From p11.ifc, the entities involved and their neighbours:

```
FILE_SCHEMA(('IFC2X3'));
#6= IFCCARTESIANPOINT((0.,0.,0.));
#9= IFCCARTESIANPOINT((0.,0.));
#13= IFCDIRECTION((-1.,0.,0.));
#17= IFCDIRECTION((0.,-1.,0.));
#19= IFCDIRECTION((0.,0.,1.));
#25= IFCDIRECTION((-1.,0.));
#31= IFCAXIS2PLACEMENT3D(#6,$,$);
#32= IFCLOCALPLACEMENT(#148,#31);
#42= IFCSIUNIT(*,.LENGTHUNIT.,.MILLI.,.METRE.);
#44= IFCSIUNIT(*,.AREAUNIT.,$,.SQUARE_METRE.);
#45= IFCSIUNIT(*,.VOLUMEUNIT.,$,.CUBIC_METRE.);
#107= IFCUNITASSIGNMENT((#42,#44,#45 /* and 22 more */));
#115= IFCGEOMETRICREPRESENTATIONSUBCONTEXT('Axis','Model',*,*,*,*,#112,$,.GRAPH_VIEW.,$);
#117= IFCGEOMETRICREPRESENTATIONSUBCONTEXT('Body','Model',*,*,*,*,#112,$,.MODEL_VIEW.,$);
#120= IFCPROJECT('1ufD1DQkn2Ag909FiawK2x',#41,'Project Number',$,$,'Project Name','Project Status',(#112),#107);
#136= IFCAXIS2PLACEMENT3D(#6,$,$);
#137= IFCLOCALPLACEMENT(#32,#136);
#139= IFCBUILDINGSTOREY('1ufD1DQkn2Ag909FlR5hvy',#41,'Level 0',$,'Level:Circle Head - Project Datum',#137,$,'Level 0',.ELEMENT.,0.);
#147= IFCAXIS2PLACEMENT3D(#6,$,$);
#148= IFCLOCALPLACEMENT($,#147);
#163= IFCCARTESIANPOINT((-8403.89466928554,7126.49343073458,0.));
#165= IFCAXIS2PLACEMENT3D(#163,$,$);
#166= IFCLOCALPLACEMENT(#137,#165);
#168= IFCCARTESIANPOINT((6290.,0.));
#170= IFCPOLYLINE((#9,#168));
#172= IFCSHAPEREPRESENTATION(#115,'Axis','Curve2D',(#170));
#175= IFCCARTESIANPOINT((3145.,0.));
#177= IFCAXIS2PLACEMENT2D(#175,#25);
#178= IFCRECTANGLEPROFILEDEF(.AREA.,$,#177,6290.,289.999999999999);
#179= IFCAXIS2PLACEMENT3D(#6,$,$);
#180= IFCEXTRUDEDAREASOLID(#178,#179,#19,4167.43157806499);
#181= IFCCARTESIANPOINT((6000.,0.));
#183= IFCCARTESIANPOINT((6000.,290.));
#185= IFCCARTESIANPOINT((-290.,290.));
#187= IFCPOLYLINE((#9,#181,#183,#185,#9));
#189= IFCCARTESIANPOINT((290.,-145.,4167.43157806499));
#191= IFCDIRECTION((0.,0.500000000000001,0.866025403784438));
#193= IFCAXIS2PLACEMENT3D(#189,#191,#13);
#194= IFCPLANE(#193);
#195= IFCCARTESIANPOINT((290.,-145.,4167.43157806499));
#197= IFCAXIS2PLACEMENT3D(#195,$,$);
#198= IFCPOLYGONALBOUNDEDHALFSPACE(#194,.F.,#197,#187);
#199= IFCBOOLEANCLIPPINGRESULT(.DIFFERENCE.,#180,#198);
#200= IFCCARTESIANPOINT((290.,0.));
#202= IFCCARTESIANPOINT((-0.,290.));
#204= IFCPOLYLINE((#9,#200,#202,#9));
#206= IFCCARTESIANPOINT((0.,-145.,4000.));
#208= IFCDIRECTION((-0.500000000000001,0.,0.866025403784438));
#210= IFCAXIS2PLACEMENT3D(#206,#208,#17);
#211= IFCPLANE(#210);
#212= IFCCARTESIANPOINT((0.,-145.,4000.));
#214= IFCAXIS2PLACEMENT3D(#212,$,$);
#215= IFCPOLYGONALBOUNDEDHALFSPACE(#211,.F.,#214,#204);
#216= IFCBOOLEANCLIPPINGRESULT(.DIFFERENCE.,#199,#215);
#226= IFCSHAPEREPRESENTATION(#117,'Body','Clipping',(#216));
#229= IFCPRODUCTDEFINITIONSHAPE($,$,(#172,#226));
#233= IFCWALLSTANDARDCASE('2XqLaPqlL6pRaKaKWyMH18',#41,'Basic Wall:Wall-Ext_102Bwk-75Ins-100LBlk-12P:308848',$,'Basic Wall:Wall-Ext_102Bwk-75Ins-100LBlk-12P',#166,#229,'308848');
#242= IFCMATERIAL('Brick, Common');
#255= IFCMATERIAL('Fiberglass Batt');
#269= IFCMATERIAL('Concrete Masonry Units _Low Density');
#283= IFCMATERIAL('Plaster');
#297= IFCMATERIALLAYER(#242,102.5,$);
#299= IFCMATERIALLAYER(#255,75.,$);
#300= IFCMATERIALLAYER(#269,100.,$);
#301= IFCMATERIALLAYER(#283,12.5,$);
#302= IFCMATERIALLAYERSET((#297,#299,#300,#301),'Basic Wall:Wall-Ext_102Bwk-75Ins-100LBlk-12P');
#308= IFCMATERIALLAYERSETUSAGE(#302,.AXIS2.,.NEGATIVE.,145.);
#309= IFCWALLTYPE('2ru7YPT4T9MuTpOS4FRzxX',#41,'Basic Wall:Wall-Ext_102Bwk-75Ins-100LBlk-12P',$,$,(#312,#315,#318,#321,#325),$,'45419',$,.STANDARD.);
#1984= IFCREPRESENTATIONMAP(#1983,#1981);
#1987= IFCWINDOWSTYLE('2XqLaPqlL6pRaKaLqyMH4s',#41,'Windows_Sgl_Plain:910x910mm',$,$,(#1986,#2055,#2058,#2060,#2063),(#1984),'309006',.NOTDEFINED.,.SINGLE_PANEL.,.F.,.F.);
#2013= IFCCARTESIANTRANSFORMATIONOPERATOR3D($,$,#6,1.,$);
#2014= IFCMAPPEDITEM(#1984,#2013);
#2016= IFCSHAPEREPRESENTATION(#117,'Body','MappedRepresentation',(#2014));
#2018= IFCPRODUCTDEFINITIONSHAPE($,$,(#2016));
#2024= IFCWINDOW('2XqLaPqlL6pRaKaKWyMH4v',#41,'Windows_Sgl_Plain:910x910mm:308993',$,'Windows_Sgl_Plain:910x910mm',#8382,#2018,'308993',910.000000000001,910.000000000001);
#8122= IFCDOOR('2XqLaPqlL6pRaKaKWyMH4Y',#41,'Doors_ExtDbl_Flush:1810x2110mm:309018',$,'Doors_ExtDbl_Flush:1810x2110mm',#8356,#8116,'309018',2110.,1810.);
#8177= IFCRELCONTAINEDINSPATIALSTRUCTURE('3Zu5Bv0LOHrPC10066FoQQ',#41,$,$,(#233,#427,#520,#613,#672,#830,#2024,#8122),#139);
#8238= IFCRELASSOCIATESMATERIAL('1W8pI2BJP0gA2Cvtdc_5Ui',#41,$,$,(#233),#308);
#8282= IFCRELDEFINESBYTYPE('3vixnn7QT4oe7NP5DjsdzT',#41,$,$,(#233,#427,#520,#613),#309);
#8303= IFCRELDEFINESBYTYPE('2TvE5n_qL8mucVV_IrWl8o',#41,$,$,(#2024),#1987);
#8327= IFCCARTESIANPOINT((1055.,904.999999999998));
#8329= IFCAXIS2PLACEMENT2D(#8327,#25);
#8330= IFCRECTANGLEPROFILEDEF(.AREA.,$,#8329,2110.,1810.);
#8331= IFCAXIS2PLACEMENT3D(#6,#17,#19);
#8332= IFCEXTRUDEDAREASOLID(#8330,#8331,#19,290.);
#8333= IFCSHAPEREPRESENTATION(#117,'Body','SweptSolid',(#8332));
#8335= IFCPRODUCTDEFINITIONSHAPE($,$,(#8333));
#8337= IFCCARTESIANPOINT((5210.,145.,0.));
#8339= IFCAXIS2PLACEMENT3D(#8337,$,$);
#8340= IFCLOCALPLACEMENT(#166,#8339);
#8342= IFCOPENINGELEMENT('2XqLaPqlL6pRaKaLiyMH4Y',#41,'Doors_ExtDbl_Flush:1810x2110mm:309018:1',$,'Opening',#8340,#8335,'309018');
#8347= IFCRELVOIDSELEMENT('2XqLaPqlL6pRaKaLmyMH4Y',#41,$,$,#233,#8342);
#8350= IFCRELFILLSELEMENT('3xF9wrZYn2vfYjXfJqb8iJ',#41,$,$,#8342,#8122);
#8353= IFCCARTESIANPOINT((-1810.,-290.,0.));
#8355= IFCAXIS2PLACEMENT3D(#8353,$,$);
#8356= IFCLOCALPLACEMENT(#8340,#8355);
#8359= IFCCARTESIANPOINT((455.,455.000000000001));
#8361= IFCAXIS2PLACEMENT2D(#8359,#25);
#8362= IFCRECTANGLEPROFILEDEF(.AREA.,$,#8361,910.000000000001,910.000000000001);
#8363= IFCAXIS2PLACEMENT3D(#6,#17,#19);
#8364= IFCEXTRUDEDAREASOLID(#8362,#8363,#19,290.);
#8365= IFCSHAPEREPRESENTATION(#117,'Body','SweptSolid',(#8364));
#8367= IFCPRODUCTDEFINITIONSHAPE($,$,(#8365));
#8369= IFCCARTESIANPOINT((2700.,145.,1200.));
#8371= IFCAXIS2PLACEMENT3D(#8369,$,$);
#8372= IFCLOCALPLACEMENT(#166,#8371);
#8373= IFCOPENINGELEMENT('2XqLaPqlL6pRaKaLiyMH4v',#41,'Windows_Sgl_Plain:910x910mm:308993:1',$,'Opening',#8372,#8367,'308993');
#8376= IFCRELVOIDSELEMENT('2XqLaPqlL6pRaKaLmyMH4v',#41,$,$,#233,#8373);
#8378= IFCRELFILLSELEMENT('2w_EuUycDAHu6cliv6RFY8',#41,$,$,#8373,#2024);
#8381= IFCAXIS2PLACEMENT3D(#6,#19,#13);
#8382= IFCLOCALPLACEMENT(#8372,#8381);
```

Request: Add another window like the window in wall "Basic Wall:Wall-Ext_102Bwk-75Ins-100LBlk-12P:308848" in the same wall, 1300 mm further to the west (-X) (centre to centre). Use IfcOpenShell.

```python
import ifcopenshell
import ifcopenshell.api.feature
import ifcopenshell.api.geometry
import ifcopenshell.api.root
import ifcopenshell.geom
import ifcopenshell.util.element
import ifcopenshell.util.placement
import ifcopenshell.util.shape
import ifcopenshell.util.unit

model = ifcopenshell.open("p11.ifc")
unit_scale = ifcopenshell.util.unit.calculate_unit_scale(model)
settings = ifcopenshell.geom.settings()


def volume(element):
    """Net volume in cubic metres, openings subtracted."""
    shape = ifcopenshell.geom.create_shape(settings, element)
    return ifcopenshell.util.shape.get_volume(shape.geometry)


def reuse_history(source, copy):
    """copy_class also copies each property set's owner history, people and application; keep the originals."""
    for rel in copy.IsDefinedBy:
        if rel.is_a("IfcRelDefinesByProperties") and (history := rel.RelatingPropertyDefinition.OwnerHistory):
            rel.RelatingPropertyDefinition.OwnerHistory = source.OwnerHistory
            ifcopenshell.util.element.remove_deep2(model, history)


window = model.by_guid("2XqLaPqlL6pRaKaKWyMH4v")
opening = window.FillsVoids[0].RelatingOpeningElement
wall = opening.VoidsElements[0].RelatingBuildingElement
before = volume(wall)
shift = ifcopenshell.util.placement.get_local_placement(wall.ObjectPlacement)[:3, 0] * -1.3 / unit_scale

# copy_class copies the void relationship, type, container and properties, but no geometry.
new_opening = ifcopenshell.api.root.copy_class(model, product=opening)
new_opening.Representation = ifcopenshell.util.element.copy_deep(
    model, opening.Representation, exclude=["IfcGeometricRepresentationContext", "IfcRepresentationMap"]
)
new_opening.Name = "Windows_Sgl_Plain:910x910mm"
new_opening.Tag = None
new_window = ifcopenshell.api.root.copy_class(model, product=window)
new_window.Representation = ifcopenshell.util.element.copy_deep(
    model, window.Representation, exclude=["IfcGeometricRepresentationContext", "IfcRepresentationMap"]
)
new_window.Name = "Windows_Sgl_Plain:910x910mm"
new_window.Tag = None
reuse_history(window, new_window)
fills = ifcopenshell.api.feature.add_filling(model, opening=new_opening, element=new_window)
fills.OwnerHistory = new_window.OwnerHistory  # required in IFC2X3

for old, new in ((opening, new_opening), (window, new_window)):
    matrix = ifcopenshell.util.placement.get_local_placement(old.ObjectPlacement)
    matrix[:3, 3] += shift
    ifcopenshell.api.geometry.edit_object_placement(model, product=new, matrix=matrix, is_si=False)

after = volume(wall)

print(f"wall volume {before:.3f} -> {after:.3f} m3")

model.write("p11_updated.ifc")
```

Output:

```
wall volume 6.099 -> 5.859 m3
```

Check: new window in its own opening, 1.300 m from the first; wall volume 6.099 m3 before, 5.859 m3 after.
